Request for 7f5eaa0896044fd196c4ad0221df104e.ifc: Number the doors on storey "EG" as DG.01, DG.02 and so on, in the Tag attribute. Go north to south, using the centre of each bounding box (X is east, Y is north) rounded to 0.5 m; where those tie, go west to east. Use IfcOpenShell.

First a look at what the model holds.

```python
import ifcopenshell
import ifcopenshell.util.element
import ifcopenshell.util.placement

model = ifcopenshell.open("7f5eaa0896044fd196c4ad0221df104e.ifc")
print(model.schema)
storey = next(s for s in model.by_type("IfcBuildingStorey") if s.Name == "EG")
doors = [e for e in ifcopenshell.util.element.get_decomposition(storey) if e.is_a("IfcDoor")]
for e in sorted(doors, key=lambda e: e.id()):
    origin = ifcopenshell.util.placement.get_local_placement(e.ObjectPlacement)[:3, 3]
    print(e.id(), e.Tag, e.Name, origin.round(2) + 0.0, sep=" | ")
```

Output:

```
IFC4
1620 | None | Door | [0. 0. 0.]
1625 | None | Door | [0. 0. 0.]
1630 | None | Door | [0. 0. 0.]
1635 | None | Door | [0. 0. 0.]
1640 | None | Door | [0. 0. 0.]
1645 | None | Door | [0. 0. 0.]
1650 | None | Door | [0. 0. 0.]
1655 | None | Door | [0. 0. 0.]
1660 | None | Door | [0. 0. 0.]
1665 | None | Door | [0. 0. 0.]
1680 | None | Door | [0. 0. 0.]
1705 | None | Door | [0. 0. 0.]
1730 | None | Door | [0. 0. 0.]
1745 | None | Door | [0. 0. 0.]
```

```python
import ifcopenshell
import ifcopenshell.geom
import ifcopenshell.util.element
import ifcopenshell.util.shape

model = ifcopenshell.open("7f5eaa0896044fd196c4ad0221df104e.ifc")
settings = ifcopenshell.geom.settings()
settings.set("use-world-coords", True)


def centre(element):
    shape = ifcopenshell.geom.create_shape(settings, element)
    return ifcopenshell.util.shape.get_bbox_centroid(shape.geometry)


storey = next(s for s in model.by_type("IfcBuildingStorey") if s.Name == "EG")
doors = [e for e in ifcopenshell.util.element.get_decomposition(storey) if e.is_a("IfcDoor")]

# Insertion points can sit at a corner or the storey origin, so sort by the geometry (in metres).
centres = {e: centre(e) for e in doors}
doors.sort(key=lambda e: (-round(centres[e][1] / 0.5), centres[e][0]))

for i, e in enumerate(doors, start=1):
    number = f"DG.{i:02d}"
    e.Tag = number
    print(e.id(), number)

model.write("7f5eaa0896044fd196c4ad0221df104e_edited.ifc")
```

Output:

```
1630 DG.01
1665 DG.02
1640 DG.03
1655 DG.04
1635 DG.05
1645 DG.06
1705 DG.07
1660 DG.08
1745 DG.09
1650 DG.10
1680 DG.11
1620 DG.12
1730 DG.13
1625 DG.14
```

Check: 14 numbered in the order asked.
